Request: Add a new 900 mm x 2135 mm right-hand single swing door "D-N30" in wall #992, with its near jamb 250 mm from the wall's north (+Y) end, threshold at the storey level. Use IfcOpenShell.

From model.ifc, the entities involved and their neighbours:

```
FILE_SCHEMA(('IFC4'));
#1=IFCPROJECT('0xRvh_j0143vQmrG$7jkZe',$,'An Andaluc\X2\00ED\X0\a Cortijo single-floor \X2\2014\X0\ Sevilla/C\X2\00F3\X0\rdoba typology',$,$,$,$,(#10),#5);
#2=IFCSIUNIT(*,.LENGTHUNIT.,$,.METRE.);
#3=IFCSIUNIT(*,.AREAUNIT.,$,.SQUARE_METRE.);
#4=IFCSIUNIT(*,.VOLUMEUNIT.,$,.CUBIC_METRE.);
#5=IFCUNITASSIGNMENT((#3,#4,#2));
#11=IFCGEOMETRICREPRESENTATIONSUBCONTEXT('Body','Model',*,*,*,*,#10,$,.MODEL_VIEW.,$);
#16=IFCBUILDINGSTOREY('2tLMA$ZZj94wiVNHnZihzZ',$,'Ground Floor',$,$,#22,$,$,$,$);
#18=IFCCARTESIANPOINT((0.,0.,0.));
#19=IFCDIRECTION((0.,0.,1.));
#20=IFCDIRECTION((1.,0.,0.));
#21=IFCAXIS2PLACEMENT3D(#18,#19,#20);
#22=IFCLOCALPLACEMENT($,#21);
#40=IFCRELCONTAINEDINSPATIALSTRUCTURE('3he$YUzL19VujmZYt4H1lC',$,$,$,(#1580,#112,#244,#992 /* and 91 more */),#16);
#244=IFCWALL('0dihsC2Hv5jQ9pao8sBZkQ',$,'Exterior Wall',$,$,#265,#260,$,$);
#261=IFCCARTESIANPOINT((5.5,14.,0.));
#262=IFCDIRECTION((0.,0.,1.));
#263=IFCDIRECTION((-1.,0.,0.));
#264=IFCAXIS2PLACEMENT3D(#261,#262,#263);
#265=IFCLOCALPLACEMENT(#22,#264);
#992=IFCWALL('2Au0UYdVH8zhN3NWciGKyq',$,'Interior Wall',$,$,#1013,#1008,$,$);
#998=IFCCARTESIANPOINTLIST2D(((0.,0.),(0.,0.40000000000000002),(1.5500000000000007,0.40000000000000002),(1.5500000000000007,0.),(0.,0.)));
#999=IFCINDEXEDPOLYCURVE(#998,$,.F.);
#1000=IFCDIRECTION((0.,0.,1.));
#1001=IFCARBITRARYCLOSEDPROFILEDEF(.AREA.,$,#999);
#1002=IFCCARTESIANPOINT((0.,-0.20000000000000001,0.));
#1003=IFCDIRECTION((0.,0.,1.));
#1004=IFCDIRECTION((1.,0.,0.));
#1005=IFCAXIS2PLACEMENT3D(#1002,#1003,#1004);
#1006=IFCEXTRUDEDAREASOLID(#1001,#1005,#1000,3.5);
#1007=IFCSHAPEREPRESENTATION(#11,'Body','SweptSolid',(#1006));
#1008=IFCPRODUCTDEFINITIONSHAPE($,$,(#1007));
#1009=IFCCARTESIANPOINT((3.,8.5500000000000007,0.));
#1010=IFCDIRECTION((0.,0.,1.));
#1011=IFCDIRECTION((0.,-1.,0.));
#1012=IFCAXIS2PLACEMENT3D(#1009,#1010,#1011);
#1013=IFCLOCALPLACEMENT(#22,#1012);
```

```python
import numpy as np
import ifcopenshell
import ifcopenshell.api.feature
import ifcopenshell.api.geometry
import ifcopenshell.api.root
import ifcopenshell.api.spatial
import ifcopenshell.geom
import ifcopenshell.util.element
import ifcopenshell.util.placement
import ifcopenshell.util.representation
import ifcopenshell.util.shape
import ifcopenshell.util.unit

model = ifcopenshell.open("model.ifc")
unit_scale = ifcopenshell.util.unit.calculate_unit_scale(model)
settings = ifcopenshell.geom.settings()


def volume(element):
    """Net volume in cubic metres, openings subtracted."""
    shape = ifcopenshell.geom.create_shape(settings, element)
    return ifcopenshell.util.shape.get_volume(shape.geometry)


wall = model.by_id(992)
storey = ifcopenshell.util.element.get_container(wall, ifc_class="IfcBuildingStorey")
context = ifcopenshell.util.representation.get_context(model, "Model", "Body", "MODEL_VIEW")
before = volume(wall)

width, height, from_end, sill = 0.9, 2.135, 0.25, 0.0  # metres

# The wall runs along its own X axis, and the end named is its -X end.
wall_shape = ifcopenshell.geom.create_shape(settings, wall)
x, y, z = ifcopenshell.util.shape.get_vertices(wall_shape.geometry).T
start = x.min() + from_end
face, thickness = float(y.min()), float(y.max() - y.min())
wall_matrix = ifcopenshell.util.placement.get_local_placement(wall.ObjectPlacement)
level = ifcopenshell.util.placement.get_local_placement(storey.ObjectPlacement)[2, 3]


def in_wall(x, y):
    """Placement at x, y metres in the wall's axes, at sill height."""
    matrix = wall_matrix.copy()
    matrix[:, 3] = wall_matrix @ np.array([x / unit_scale, y / unit_scale, 0.0, 1.0])
    matrix[2, 3] = level + sill / unit_scale
    return matrix


# Opening: a box that overshoots both wall faces by 50 mm.
opening = ifcopenshell.api.root.create_entity(model, ifc_class="IfcOpeningElement", predefined_type="OPENING")
box = ifcopenshell.api.geometry.add_wall_representation(
    model, context=context, length=width, height=height, thickness=thickness + 0.1
)
ifcopenshell.api.geometry.assign_representation(model, product=opening, representation=box)
ifcopenshell.api.geometry.edit_object_placement(model, product=opening, matrix=in_wall(start, face - 0.05), is_si=False)
ifcopenshell.api.feature.add_feature(model, feature=opening, element=wall)

door = ifcopenshell.api.root.create_entity(model, ifc_class="IfcDoor", name="D-N30", predefined_type="DOOR")
door.OverallWidth, door.OverallHeight = width / unit_scale, height / unit_scale
door.OperationType = "SINGLE_SWING_RIGHT"
body = ifcopenshell.api.geometry.add_door_representation(
    model,
    context=context,
    overall_width=door.OverallWidth,
    overall_height=door.OverallHeight,
    operation_type="SINGLE_SWING_RIGHT",
    lining_properties={"LiningDepth": thickness / unit_scale, "ThresholdDepth": thickness / unit_scale},
)
ifcopenshell.api.geometry.assign_representation(model, product=door, representation=body)
ifcopenshell.api.spatial.assign_container(model, products=[door], relating_structure=storey)
ifcopenshell.api.feature.add_filling(model, opening=opening, element=door)

# The lining spans the wall, so the door starts at the wall face.
ifcopenshell.api.geometry.edit_object_placement(model, product=door, matrix=in_wall(start, face), is_si=False)

after = volume(wall)

print(f"wall volume {before:.3f} -> {after:.3f} m3")

model.write("model_v2.ifc")
```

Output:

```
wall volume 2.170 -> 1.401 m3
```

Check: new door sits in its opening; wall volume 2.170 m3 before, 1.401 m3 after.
